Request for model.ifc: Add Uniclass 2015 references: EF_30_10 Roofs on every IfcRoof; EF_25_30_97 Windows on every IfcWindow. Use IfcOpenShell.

First a look at what the model holds.

```python
import ifcopenshell

model = ifcopenshell.open("model.ifc")
print(model.schema)
print("classifications:", [c.Name for c in model.by_type("IfcClassification")])
for ifc_class in ("IfcDoor", "IfcRoof", "IfcStair", "IfcWall", "IfcWindow"):
    print(ifc_class, len(model.by_type(ifc_class)))
```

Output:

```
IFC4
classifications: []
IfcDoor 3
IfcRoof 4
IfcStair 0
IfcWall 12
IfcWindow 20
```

```python
import ifcopenshell
import ifcopenshell.api.classification

model = ifcopenshell.open("model.ifc")

system = ifcopenshell.api.classification.add_classification(model, classification="Uniclass 2015")

codes = {
    "IfcRoof": ("EF_30_10", "Roofs"),
    "IfcWindow": ("EF_25_30_97", "Windows"),
}
for ifc_class, (code, name) in codes.items():
    products = model.by_type(ifc_class)
    ifcopenshell.api.classification.add_reference(
        model, products=products, classification=system, identification=code, name=name
    )
    print(code, len(products))

model.write("model_v2.ifc")
```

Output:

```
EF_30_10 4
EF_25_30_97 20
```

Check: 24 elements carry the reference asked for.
